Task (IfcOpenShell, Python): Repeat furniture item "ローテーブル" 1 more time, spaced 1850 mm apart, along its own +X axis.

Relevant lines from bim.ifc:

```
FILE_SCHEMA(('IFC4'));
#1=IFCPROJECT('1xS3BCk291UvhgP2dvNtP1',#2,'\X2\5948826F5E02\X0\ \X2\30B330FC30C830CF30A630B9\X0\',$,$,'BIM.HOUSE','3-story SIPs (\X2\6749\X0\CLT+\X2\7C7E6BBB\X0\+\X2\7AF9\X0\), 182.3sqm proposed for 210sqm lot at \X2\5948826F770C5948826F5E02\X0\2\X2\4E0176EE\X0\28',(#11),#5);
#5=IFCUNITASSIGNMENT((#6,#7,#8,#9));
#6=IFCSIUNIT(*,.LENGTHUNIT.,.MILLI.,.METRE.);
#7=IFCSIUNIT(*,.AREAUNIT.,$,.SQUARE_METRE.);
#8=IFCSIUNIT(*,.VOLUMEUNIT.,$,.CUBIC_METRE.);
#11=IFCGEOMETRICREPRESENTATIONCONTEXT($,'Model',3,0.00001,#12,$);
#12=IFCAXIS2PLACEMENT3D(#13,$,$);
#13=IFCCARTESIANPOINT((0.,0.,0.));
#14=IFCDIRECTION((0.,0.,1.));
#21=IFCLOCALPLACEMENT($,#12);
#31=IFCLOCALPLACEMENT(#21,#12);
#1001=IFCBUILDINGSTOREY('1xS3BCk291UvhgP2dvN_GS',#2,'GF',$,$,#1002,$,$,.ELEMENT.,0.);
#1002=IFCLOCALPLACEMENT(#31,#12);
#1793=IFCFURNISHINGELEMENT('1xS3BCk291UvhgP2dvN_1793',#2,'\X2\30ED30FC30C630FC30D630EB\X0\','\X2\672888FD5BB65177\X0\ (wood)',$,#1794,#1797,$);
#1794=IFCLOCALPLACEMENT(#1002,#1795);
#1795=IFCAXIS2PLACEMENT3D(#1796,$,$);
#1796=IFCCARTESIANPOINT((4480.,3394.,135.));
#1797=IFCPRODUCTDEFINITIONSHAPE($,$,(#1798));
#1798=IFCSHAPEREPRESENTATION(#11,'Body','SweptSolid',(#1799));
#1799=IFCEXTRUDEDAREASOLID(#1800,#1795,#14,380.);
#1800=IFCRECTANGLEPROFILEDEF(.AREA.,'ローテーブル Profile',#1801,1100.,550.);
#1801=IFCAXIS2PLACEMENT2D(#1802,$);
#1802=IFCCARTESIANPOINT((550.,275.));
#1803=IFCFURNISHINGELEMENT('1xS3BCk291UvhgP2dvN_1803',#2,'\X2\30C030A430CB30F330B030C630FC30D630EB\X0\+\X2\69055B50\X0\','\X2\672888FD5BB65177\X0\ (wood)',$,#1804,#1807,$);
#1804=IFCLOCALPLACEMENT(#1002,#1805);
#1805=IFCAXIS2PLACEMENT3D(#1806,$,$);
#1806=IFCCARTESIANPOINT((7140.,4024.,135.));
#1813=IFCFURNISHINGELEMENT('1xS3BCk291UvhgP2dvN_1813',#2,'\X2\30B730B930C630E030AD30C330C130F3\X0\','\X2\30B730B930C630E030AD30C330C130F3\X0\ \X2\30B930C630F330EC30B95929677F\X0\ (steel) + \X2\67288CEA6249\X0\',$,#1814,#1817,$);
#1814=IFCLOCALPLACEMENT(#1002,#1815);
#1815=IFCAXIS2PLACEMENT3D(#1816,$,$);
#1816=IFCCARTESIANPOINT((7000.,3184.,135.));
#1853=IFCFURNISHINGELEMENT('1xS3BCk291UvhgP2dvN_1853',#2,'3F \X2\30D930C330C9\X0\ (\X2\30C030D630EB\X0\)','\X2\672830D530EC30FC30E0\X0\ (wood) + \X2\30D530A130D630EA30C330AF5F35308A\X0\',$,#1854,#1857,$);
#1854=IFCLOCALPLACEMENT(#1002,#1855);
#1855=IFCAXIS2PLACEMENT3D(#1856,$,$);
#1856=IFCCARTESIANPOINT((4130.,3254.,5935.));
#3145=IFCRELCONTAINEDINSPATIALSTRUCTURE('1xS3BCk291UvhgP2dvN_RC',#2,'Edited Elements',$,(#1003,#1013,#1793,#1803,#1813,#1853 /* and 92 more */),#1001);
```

```python
import ifcopenshell
import ifcopenshell.api.geometry
import ifcopenshell.api.root
import ifcopenshell.util.element
import ifcopenshell.util.placement

model = ifcopenshell.open("bim.ifc")


def reuse_history(source, copy):
    """copy_class also copies each property set's owner history, people and application; keep the originals."""
    for rel in copy.IsDefinedBy:
        if rel.is_a("IfcRelDefinesByProperties") and (history := rel.RelatingPropertyDefinition.OwnerHistory):
            rel.RelatingPropertyDefinition.OwnerHistory = source.OwnerHistory
            ifcopenshell.util.element.remove_deep2(model, history)


source = model.by_guid("1xS3BCk291UvhgP2dvN_1793")
base = ifcopenshell.util.placement.get_local_placement(source.ObjectPlacement)
step = base[:3, 0] * 1850.0

for i in range(1, 2):
    copy = ifcopenshell.api.root.copy_class(model, product=source)
    copy.Representation = ifcopenshell.util.element.copy_deep(
        model, source.Representation, exclude=["IfcGeometricRepresentationContext", "IfcRepresentationMap"]
    )
    reuse_history(source, copy)
    matrix = base.copy()
    matrix[:3, 3] += i * step
    print("added at", matrix[:3, 3].round(3) + 0.0)
    ifcopenshell.api.geometry.edit_object_placement(model, product=copy, matrix=matrix, is_si=False)

model.write("bim_updated.ifc")
```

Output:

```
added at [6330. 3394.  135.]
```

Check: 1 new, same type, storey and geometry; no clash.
